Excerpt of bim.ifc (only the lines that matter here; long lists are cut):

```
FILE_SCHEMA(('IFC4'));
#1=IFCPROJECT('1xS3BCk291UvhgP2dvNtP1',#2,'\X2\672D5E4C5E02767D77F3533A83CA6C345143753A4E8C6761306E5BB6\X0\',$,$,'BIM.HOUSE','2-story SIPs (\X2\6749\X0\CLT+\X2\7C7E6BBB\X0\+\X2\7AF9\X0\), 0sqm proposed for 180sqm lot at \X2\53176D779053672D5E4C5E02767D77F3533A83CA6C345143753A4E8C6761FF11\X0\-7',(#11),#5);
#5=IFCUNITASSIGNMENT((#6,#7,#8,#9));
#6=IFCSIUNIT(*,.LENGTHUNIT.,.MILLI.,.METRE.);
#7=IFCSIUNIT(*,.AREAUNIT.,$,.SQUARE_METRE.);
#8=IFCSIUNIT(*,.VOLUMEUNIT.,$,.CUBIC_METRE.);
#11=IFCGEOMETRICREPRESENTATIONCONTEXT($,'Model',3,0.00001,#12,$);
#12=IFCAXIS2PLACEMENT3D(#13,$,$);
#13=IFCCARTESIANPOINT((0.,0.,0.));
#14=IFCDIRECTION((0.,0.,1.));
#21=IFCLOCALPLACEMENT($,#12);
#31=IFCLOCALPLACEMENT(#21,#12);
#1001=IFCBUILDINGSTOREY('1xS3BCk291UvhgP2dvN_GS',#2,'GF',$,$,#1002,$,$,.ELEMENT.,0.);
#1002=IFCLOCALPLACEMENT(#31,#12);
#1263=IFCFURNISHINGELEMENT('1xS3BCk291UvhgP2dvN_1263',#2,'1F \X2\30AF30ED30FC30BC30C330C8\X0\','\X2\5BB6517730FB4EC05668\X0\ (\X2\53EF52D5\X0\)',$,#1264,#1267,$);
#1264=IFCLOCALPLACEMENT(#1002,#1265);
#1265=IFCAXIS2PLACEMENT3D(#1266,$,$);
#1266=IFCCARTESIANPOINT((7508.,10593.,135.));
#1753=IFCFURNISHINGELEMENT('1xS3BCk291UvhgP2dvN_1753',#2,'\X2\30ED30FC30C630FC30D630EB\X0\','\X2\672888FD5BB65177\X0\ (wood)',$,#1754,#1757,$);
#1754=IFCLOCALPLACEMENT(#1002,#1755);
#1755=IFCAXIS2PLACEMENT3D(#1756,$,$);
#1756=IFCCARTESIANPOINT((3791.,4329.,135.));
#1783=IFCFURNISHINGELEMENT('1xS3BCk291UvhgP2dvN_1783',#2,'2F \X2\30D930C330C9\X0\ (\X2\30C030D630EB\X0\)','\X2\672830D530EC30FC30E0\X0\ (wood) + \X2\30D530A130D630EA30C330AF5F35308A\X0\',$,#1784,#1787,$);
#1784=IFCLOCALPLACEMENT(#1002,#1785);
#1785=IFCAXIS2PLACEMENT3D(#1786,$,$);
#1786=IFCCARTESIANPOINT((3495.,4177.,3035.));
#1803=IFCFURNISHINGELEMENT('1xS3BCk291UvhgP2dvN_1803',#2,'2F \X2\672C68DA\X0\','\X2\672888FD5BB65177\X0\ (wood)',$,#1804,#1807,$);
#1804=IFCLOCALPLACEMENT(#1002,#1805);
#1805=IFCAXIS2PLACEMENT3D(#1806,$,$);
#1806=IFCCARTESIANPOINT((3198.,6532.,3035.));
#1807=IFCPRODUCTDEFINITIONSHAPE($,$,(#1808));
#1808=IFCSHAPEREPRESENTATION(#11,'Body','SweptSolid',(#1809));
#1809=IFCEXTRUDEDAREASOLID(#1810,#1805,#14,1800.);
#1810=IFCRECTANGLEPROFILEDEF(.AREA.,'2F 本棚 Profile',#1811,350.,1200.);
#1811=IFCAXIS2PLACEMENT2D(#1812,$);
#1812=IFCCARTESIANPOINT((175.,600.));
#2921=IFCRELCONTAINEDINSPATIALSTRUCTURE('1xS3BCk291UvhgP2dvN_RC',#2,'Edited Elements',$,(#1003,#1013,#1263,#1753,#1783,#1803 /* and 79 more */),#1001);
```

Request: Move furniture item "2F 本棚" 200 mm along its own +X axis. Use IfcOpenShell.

```python
import ifcopenshell
import ifcopenshell.api.geometry
import ifcopenshell.util.placement

model = ifcopenshell.open("bim.ifc")

item = model.by_guid("1xS3BCk291UvhgP2dvN_1803")
matrix = ifcopenshell.util.placement.get_local_placement(item.ObjectPlacement)
matrix[:3, 3] += matrix[:3, 0] * 200.0
ifcopenshell.api.geometry.edit_object_placement(model, product=item, matrix=matrix, is_si=False)

print(ifcopenshell.util.placement.get_local_placement(item.ObjectPlacement).round(3) + 0.0)

model.write("bim_rev.ifc")
```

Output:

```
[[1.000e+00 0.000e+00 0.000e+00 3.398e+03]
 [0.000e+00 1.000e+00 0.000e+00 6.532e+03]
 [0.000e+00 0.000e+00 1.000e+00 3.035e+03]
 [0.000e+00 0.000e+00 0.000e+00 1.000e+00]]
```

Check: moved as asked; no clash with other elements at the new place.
